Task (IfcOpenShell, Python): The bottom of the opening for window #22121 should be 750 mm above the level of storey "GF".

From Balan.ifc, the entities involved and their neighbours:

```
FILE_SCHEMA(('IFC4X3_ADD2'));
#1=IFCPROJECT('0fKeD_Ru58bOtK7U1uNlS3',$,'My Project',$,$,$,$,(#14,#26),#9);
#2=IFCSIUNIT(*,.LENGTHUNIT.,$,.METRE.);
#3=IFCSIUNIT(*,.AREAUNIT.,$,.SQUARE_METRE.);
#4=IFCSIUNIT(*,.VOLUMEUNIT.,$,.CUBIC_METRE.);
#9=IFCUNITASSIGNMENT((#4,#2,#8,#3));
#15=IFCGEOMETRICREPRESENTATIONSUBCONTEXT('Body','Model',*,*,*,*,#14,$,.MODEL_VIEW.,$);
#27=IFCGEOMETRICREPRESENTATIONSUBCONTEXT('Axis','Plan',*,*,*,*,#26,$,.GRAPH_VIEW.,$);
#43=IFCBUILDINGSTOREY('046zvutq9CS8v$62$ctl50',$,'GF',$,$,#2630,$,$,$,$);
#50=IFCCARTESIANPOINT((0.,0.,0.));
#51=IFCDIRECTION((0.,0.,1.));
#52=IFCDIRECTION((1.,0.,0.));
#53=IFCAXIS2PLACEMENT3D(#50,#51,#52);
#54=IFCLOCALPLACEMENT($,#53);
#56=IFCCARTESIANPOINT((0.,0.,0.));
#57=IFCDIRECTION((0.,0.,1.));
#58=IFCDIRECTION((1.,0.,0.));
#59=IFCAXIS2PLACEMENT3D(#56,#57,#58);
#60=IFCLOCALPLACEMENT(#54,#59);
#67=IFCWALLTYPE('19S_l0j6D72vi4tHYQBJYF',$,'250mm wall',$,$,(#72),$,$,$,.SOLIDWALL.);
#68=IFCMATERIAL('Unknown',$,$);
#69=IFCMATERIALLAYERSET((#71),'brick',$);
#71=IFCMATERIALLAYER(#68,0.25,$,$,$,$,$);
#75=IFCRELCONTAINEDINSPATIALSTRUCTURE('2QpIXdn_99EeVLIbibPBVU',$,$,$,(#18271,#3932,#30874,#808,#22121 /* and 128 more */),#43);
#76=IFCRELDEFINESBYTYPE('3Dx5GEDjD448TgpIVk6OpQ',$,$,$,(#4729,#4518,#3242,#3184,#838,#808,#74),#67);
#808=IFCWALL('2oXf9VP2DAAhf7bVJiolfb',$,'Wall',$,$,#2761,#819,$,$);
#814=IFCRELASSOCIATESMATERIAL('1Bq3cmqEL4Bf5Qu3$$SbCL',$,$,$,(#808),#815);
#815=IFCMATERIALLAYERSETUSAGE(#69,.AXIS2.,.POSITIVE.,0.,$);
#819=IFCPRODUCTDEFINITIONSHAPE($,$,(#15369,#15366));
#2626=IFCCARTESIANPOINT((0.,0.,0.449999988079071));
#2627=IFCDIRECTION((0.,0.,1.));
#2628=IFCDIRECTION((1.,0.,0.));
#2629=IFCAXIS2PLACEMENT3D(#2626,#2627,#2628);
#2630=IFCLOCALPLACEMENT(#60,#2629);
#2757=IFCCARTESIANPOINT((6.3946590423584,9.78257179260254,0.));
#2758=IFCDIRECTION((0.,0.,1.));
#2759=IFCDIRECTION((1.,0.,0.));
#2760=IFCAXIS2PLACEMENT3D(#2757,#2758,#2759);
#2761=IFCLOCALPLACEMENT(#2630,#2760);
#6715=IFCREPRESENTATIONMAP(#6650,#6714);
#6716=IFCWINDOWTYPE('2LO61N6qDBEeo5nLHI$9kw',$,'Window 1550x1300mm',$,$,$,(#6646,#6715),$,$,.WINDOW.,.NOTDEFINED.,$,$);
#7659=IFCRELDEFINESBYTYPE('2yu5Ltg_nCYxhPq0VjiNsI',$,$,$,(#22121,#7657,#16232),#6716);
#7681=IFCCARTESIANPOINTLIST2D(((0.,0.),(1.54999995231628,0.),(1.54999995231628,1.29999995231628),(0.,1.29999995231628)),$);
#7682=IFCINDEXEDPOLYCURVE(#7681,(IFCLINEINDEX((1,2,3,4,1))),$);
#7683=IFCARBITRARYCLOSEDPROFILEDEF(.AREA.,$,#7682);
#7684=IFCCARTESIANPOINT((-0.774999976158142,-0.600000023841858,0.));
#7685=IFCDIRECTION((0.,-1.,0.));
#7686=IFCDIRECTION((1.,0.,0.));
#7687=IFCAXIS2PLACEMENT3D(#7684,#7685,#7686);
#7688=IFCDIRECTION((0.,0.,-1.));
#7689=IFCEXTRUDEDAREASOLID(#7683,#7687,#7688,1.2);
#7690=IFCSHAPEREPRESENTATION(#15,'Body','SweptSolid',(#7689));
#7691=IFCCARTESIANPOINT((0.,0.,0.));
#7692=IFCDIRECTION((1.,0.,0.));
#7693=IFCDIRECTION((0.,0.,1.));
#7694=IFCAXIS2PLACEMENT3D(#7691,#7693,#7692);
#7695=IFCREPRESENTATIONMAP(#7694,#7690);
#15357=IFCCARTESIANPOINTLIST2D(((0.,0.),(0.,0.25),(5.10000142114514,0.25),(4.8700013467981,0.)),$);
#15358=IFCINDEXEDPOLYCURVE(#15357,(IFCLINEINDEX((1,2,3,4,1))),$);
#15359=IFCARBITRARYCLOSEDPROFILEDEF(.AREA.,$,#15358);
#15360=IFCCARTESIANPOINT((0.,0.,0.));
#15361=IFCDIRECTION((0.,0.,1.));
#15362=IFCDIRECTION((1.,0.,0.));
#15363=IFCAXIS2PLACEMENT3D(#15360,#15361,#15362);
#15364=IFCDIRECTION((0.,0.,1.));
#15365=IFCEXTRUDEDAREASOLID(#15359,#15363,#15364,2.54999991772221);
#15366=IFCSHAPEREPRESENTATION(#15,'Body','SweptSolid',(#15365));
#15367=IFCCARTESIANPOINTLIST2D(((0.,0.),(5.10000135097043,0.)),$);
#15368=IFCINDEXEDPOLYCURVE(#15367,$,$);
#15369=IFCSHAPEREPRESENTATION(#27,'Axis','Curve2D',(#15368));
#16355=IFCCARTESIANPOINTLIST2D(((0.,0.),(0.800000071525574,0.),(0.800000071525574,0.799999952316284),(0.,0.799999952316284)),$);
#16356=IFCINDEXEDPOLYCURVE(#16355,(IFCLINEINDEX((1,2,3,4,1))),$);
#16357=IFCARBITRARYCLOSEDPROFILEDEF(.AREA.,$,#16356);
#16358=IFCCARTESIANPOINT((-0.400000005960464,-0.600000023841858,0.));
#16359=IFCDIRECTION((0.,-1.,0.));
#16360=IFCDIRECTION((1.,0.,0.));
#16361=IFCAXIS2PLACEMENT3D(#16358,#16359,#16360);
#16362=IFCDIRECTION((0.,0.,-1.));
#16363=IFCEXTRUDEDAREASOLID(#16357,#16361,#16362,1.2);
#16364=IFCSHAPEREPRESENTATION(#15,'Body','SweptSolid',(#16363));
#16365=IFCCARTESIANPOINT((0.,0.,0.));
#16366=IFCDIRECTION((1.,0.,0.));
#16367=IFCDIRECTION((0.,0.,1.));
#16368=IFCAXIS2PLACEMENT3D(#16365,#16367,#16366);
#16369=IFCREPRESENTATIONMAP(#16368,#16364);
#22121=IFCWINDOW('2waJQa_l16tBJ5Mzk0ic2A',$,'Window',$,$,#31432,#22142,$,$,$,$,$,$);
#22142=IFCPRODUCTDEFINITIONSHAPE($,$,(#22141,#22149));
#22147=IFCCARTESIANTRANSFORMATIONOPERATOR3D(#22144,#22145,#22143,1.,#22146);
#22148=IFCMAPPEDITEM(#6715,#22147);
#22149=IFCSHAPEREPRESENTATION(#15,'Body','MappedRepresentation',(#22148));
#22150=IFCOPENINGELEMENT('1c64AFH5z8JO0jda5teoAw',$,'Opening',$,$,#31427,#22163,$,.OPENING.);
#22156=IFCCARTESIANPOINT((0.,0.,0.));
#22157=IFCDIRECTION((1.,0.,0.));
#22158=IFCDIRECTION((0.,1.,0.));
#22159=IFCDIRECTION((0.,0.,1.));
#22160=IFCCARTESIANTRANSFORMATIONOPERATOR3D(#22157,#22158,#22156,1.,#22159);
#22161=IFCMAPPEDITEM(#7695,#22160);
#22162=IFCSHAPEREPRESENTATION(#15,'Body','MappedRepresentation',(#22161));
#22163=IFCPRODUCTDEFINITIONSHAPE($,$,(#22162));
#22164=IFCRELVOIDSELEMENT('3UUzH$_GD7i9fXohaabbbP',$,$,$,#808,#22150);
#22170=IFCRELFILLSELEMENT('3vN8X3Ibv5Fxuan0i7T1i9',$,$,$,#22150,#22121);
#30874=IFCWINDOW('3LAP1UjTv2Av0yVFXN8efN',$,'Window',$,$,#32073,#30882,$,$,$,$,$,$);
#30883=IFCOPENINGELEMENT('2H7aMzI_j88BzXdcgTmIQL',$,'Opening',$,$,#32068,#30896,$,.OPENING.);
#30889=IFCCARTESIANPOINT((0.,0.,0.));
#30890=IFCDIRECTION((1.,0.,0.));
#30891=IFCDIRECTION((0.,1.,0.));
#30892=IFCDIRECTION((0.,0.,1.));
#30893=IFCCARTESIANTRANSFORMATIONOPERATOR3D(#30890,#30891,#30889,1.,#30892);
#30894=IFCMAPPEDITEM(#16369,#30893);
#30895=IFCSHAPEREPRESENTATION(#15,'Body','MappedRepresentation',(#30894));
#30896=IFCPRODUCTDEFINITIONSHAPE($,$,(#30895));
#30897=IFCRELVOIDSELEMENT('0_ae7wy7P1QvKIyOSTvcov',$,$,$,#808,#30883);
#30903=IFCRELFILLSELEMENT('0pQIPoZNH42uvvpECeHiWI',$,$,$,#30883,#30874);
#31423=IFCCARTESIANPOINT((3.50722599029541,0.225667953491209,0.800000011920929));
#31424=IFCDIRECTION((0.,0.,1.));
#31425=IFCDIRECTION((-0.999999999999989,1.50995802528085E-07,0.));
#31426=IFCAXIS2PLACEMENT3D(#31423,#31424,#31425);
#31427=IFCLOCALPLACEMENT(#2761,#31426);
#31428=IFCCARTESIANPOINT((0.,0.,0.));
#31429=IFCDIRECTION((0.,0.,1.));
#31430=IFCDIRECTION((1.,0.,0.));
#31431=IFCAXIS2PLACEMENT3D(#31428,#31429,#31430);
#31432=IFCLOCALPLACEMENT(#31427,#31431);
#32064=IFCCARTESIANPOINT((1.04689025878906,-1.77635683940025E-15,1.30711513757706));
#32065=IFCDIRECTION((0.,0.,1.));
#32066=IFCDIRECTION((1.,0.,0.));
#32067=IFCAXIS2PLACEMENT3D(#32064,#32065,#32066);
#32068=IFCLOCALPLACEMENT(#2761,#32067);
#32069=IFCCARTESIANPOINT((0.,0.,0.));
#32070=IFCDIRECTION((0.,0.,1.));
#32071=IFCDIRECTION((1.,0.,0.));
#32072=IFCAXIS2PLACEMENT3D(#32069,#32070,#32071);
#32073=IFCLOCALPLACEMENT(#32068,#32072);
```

```python
import numpy as np
import ifcopenshell
import ifcopenshell.api.geometry
import ifcopenshell.geom
import ifcopenshell.util.element
import ifcopenshell.util.placement
import ifcopenshell.util.shape
import ifcopenshell.util.unit

model = ifcopenshell.open("Balan.ifc")
unit_scale = ifcopenshell.util.unit.calculate_unit_scale(model)

window = model.by_guid("2waJQa_l16tBJ5Mzk0ic2A")
opening = window.FillsVoids[0].RelatingOpeningElement
storey = ifcopenshell.util.element.get_container(window, ifc_class="IfcBuildingStorey")
level = ifcopenshell.util.placement.get_local_placement(storey.ObjectPlacement)[2, 3]

# The opening's origin need not be at the sill, so measure its lowest point.
shape = ifcopenshell.geom.create_shape(ifcopenshell.geom.settings(), opening)
bottom = ifcopenshell.util.shape.get_shape_bottom_elevation(shape, shape.geometry) / unit_scale
dz = level + 0.75 - bottom

shift = np.array([0.0, 0.0, dz])
# The window is placed relative to its opening, so it follows when the opening moves.
matrix = ifcopenshell.util.placement.get_local_placement(opening.ObjectPlacement)
matrix[:3, 3] += shift
ifcopenshell.api.geometry.edit_object_placement(
    model, product=opening, matrix=matrix, is_si=False, should_transform_children=True
)

print(f"moved by {dz * unit_scale:+.3f} m")

model.write("Balan_updated.ifc")
```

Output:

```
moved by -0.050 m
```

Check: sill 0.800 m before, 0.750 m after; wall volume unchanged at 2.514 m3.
